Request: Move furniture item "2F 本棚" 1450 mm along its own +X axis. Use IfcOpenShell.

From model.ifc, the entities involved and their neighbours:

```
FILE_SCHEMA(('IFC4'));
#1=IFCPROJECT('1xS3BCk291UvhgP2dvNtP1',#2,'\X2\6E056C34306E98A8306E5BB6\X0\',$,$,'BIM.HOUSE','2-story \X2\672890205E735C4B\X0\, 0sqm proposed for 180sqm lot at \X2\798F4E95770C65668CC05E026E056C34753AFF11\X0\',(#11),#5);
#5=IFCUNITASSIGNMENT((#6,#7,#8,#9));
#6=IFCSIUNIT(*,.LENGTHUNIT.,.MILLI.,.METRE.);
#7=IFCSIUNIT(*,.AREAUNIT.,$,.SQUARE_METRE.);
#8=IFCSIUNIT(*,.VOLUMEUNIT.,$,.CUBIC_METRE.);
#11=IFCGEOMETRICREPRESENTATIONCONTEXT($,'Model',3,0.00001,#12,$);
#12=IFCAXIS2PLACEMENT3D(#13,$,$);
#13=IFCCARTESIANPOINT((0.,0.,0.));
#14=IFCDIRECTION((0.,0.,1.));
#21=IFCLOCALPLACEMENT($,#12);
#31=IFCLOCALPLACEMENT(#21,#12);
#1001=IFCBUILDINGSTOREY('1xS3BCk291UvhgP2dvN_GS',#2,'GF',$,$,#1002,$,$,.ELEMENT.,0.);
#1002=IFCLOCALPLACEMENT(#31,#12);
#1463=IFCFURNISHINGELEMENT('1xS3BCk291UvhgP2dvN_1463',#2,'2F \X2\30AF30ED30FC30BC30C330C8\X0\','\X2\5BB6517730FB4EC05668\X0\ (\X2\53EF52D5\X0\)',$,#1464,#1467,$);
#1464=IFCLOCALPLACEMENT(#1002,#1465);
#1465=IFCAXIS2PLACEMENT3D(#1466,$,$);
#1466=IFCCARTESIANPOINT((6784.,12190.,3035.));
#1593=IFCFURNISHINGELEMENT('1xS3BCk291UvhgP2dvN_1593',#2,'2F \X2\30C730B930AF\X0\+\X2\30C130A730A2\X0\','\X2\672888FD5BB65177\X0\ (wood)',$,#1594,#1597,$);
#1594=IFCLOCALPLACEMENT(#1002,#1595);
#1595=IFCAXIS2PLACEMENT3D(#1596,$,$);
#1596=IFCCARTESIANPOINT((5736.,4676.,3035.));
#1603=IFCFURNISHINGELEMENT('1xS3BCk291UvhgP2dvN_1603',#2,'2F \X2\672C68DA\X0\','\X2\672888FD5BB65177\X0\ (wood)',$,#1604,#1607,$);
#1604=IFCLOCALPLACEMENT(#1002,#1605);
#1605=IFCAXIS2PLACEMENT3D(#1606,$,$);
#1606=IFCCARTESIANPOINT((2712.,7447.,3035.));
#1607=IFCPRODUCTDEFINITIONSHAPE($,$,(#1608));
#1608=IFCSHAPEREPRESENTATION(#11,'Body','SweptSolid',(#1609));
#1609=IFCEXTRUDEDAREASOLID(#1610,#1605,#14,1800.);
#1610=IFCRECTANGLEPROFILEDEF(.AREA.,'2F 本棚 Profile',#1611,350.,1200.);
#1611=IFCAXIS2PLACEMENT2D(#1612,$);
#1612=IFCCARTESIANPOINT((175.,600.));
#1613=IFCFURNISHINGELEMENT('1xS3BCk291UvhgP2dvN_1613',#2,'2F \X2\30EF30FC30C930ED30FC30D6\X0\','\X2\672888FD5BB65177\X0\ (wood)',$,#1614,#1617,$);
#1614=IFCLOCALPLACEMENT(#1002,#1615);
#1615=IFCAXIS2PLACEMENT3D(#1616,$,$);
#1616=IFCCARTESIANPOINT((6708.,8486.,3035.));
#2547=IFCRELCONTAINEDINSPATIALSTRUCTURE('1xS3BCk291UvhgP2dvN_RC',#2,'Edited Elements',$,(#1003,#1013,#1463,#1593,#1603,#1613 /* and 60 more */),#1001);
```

```python
import ifcopenshell
import ifcopenshell.api.geometry
import ifcopenshell.util.placement
import ifcopenshell.util.unit

model = ifcopenshell.open("model.ifc")
unit_scale = ifcopenshell.util.unit.calculate_unit_scale(model)

item = model.by_guid("1xS3BCk291UvhgP2dvN_1603")
matrix = ifcopenshell.util.placement.get_local_placement(item.ObjectPlacement)
matrix[:3, 3] += matrix[:3, 0] * 1.45 / unit_scale
ifcopenshell.api.geometry.edit_object_placement(model, product=item, matrix=matrix, is_si=False)

print(ifcopenshell.util.placement.get_local_placement(item.ObjectPlacement).round(3) + 0.0)

model.write("model_rev.ifc")
```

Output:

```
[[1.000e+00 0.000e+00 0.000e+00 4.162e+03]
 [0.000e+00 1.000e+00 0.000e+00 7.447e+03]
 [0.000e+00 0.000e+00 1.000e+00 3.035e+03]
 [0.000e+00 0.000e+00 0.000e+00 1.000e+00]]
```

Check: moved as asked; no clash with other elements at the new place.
